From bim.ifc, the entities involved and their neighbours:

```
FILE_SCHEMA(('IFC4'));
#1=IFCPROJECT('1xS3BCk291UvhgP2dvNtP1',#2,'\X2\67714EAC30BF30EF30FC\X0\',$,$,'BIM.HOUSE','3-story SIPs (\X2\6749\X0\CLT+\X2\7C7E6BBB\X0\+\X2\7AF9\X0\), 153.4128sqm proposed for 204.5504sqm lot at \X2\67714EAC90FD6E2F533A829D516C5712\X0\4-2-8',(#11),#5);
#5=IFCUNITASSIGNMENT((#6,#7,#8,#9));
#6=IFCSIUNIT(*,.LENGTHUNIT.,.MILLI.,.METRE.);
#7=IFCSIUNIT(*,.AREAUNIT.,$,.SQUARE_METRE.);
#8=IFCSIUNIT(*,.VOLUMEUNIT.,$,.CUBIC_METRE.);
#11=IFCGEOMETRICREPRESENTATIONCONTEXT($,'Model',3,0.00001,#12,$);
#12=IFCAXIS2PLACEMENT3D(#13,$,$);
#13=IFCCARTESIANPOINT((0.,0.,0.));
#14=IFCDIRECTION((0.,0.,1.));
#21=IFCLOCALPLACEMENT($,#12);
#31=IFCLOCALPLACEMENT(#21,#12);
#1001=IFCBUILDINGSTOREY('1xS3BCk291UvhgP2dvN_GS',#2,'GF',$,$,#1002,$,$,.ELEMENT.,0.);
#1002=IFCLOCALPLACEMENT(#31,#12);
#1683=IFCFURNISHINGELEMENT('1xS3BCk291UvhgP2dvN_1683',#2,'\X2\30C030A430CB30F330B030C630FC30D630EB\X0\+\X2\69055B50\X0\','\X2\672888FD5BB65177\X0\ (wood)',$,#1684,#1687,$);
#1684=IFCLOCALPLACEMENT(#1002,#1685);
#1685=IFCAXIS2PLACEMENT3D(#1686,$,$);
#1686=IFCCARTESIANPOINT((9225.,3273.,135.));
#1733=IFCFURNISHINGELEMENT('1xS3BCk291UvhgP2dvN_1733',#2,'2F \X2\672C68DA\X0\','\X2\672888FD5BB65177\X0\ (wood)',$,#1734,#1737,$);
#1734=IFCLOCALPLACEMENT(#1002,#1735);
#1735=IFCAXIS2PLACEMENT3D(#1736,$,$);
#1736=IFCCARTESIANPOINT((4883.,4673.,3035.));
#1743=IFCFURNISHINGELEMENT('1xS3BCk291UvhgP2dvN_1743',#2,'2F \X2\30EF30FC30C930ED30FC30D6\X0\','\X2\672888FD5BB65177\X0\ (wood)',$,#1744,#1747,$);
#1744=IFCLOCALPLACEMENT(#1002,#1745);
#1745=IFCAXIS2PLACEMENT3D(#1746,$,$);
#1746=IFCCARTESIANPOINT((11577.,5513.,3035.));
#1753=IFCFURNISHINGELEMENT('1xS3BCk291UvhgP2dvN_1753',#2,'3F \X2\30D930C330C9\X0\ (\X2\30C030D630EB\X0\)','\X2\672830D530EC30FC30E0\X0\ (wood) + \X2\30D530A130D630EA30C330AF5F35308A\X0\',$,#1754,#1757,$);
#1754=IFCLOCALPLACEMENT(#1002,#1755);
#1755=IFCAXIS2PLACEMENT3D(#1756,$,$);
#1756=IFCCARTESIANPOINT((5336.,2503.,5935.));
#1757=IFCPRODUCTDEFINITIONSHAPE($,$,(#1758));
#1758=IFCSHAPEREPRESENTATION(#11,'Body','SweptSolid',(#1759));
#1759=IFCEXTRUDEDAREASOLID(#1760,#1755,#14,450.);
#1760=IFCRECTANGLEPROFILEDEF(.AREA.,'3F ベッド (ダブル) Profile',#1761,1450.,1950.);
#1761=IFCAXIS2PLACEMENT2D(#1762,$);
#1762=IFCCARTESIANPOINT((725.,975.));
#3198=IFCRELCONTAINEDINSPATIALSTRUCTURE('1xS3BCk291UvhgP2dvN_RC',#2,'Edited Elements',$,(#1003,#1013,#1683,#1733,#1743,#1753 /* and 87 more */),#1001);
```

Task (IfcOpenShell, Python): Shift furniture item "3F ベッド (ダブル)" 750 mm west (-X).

```python
import ifcopenshell
import ifcopenshell.api.geometry
import ifcopenshell.util.placement
import ifcopenshell.util.unit

model = ifcopenshell.open("bim.ifc")
unit_scale = ifcopenshell.util.unit.calculate_unit_scale(model)

item = model.by_guid("1xS3BCk291UvhgP2dvN_1753")
matrix = ifcopenshell.util.placement.get_local_placement(item.ObjectPlacement)
matrix[0, 3] -= 0.75 / unit_scale
ifcopenshell.api.geometry.edit_object_placement(model, product=item, matrix=matrix, is_si=False)

print(ifcopenshell.util.placement.get_local_placement(item.ObjectPlacement).round(3) + 0.0)

model.write("bim_v2.ifc")
```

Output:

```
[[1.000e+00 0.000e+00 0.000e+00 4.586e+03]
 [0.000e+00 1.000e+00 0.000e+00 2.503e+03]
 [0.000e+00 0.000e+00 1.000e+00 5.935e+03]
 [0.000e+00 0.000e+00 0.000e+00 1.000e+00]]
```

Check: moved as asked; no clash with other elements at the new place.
